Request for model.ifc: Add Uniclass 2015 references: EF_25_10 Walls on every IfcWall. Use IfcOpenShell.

First a look at what the model holds.

```python
import ifcopenshell

model = ifcopenshell.open("model.ifc")
print(model.schema)
print("classifications:", [c.Name for c in model.by_type("IfcClassification")])
for ifc_class in ("IfcDoor", "IfcRoof", "IfcStair", "IfcWall", "IfcWindow"):
    print(ifc_class, len(model.by_type(ifc_class)))
```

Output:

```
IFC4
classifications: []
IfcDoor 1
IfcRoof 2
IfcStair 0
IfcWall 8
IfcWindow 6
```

```python
import ifcopenshell
import ifcopenshell.api.classification

model = ifcopenshell.open("model.ifc")

system = ifcopenshell.api.classification.add_classification(model, classification="Uniclass 2015")

codes = {
    "IfcWall": ("EF_25_10", "Walls"),
}
for ifc_class, (code, name) in codes.items():
    products = model.by_type(ifc_class)
    ifcopenshell.api.classification.add_reference(
        model, products=products, classification=system, identification=code, name=name
    )
    print(code, len(products))

model.write("model_rev.ifc")
```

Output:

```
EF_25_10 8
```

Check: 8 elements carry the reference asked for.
